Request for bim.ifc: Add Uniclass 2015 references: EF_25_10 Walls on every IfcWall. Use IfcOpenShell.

First a look at what the model holds.

```python
import ifcopenshell

model = ifcopenshell.open("bim.ifc")
print(model.schema)
print("classifications:", [c.Name for c in model.by_type("IfcClassification")])
for ifc_class in ("IfcDoor", "IfcRoof", "IfcStair", "IfcWall", "IfcWindow"):
    print(ifc_class, len(model.by_type(ifc_class)))
```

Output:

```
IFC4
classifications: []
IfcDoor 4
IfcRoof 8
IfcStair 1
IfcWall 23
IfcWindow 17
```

```python
import ifcopenshell
import ifcopenshell.api.classification

model = ifcopenshell.open("bim.ifc")

system = ifcopenshell.api.classification.add_classification(model, classification="Uniclass 2015")

codes = {
    "IfcWall": ("EF_25_10", "Walls"),
}
for ifc_class, (code, name) in codes.items():
    products = model.by_type(ifc_class)
    ifcopenshell.api.classification.add_reference(
        model, products=products, classification=system, identification=code, name=name
    )
    print(code, len(products))

model.write("bim_v2.ifc")
```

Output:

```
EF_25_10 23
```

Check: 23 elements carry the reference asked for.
